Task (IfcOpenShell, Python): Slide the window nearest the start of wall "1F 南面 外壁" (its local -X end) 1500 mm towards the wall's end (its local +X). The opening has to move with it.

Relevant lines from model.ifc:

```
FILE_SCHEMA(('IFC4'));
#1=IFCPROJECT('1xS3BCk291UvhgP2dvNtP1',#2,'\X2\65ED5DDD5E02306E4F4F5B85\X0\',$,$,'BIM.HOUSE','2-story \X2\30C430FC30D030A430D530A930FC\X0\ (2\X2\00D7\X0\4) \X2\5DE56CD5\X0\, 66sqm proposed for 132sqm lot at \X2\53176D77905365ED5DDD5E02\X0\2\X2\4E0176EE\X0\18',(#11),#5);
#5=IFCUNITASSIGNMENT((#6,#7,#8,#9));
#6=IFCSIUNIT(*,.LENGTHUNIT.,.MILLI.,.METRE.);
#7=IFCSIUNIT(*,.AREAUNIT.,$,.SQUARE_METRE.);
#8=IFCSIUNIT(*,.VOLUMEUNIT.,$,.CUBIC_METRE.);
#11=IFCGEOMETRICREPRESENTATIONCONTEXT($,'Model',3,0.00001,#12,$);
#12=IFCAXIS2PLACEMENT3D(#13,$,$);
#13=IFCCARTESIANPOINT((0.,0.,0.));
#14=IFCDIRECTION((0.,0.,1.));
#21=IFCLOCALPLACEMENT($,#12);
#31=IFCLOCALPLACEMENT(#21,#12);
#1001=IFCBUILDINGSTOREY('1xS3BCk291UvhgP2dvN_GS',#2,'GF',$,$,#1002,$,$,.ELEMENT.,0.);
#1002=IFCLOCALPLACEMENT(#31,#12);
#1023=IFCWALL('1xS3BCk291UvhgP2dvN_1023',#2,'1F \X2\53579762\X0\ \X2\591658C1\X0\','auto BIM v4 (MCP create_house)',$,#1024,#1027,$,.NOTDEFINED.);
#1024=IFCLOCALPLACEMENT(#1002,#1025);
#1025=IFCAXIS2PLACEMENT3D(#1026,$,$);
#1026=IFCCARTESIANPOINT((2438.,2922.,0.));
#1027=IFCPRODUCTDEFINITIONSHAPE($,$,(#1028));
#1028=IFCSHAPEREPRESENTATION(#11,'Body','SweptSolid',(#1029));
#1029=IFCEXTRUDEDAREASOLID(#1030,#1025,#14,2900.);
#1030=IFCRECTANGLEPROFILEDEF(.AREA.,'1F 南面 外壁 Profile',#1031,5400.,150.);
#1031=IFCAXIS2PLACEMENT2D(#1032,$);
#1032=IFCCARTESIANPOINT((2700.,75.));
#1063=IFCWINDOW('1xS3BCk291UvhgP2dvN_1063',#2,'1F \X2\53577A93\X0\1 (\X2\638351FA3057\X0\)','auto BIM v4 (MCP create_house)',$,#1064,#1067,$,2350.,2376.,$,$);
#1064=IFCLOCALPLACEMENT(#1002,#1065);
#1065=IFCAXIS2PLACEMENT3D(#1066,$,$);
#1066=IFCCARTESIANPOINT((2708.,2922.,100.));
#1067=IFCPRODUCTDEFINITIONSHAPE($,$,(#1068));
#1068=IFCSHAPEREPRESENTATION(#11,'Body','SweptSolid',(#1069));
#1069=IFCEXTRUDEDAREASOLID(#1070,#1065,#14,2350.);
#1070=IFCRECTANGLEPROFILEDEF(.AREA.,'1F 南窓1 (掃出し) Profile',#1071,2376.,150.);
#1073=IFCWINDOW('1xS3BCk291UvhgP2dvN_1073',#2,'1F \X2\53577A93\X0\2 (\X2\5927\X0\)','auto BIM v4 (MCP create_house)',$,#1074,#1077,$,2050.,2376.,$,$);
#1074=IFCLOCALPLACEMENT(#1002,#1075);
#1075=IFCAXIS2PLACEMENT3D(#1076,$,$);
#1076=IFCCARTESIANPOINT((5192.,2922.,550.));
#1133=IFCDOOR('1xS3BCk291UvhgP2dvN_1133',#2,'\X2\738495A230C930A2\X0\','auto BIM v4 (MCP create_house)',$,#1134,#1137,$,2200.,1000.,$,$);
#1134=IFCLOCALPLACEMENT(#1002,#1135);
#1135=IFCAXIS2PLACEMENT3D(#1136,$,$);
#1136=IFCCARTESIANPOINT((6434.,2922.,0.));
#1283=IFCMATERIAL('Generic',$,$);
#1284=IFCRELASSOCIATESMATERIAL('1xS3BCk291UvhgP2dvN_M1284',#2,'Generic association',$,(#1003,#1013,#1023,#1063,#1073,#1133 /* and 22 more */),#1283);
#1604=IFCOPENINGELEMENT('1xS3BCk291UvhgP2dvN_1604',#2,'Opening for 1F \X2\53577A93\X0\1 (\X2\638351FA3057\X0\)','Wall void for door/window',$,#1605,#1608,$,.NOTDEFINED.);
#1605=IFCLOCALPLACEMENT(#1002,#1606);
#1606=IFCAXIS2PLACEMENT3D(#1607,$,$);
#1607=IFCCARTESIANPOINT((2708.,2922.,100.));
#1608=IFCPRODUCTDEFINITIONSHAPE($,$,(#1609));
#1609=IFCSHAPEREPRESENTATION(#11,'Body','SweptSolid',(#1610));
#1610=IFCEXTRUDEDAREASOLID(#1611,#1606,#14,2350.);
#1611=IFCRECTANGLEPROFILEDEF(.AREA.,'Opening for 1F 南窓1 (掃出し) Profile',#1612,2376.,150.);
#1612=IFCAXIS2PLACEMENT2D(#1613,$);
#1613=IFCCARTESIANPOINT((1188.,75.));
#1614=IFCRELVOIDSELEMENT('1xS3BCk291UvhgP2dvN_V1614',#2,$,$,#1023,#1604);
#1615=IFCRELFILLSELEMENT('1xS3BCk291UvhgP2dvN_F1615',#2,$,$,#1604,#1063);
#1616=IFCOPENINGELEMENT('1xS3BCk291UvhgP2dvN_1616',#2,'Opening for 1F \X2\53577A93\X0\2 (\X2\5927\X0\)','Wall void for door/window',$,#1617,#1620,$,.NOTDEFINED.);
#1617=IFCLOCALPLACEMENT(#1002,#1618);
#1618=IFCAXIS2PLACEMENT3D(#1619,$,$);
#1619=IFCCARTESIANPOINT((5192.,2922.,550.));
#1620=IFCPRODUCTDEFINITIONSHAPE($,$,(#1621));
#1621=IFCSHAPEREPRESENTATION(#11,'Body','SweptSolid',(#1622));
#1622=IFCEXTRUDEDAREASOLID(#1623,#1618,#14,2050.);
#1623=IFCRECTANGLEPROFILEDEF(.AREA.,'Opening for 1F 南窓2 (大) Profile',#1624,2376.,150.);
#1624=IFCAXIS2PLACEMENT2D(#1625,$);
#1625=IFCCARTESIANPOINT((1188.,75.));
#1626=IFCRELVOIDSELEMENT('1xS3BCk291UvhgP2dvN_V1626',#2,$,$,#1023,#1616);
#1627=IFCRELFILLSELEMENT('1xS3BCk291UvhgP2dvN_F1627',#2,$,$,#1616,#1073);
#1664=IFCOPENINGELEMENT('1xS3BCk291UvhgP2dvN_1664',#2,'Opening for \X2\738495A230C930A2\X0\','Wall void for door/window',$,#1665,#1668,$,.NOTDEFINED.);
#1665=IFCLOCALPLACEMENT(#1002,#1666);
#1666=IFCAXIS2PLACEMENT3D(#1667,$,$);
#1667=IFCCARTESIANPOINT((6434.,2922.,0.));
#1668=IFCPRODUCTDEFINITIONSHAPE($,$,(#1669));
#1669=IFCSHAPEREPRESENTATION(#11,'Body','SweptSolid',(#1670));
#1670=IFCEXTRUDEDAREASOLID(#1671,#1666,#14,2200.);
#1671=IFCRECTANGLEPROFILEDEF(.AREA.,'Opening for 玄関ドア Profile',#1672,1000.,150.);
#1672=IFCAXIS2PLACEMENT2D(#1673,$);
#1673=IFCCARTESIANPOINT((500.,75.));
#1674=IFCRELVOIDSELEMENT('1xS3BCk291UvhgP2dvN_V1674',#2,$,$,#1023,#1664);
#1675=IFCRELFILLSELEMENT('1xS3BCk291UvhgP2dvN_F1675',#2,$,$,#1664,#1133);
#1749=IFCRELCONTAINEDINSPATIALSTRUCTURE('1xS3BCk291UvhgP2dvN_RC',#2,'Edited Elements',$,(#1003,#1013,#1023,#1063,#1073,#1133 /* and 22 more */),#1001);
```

```python
import ifcopenshell
import ifcopenshell.api.geometry
import ifcopenshell.util.placement
import ifcopenshell.util.unit

model = ifcopenshell.open("model.ifc")
unit_scale = ifcopenshell.util.unit.calculate_unit_scale(model)

window = model.by_guid("1xS3BCk291UvhgP2dvN_1063")
opening = window.FillsVoids[0].RelatingOpeningElement
wall = opening.VoidsElements[0].RelatingBuildingElement

wall_matrix = ifcopenshell.util.placement.get_local_placement(wall.ObjectPlacement)
shift = wall_matrix[:3, 0] * 1.5 / unit_scale
before = ifcopenshell.util.placement.get_local_placement(window.ObjectPlacement)[:3, 3].copy()

# The window is not placed relative to its opening, so move both.
for product in (opening, window):
    matrix = ifcopenshell.util.placement.get_local_placement(product.ObjectPlacement)
    matrix[:3, 3] += shift
    ifcopenshell.api.geometry.edit_object_placement(model, product=product, matrix=matrix, is_si=False)

after = ifcopenshell.util.placement.get_local_placement(window.ObjectPlacement)[:3, 3]
print("window moved by", (after - before).round(3) + 0.0)

model.write("model-out.ifc")
```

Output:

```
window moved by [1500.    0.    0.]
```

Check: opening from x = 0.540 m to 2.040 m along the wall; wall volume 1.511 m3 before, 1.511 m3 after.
